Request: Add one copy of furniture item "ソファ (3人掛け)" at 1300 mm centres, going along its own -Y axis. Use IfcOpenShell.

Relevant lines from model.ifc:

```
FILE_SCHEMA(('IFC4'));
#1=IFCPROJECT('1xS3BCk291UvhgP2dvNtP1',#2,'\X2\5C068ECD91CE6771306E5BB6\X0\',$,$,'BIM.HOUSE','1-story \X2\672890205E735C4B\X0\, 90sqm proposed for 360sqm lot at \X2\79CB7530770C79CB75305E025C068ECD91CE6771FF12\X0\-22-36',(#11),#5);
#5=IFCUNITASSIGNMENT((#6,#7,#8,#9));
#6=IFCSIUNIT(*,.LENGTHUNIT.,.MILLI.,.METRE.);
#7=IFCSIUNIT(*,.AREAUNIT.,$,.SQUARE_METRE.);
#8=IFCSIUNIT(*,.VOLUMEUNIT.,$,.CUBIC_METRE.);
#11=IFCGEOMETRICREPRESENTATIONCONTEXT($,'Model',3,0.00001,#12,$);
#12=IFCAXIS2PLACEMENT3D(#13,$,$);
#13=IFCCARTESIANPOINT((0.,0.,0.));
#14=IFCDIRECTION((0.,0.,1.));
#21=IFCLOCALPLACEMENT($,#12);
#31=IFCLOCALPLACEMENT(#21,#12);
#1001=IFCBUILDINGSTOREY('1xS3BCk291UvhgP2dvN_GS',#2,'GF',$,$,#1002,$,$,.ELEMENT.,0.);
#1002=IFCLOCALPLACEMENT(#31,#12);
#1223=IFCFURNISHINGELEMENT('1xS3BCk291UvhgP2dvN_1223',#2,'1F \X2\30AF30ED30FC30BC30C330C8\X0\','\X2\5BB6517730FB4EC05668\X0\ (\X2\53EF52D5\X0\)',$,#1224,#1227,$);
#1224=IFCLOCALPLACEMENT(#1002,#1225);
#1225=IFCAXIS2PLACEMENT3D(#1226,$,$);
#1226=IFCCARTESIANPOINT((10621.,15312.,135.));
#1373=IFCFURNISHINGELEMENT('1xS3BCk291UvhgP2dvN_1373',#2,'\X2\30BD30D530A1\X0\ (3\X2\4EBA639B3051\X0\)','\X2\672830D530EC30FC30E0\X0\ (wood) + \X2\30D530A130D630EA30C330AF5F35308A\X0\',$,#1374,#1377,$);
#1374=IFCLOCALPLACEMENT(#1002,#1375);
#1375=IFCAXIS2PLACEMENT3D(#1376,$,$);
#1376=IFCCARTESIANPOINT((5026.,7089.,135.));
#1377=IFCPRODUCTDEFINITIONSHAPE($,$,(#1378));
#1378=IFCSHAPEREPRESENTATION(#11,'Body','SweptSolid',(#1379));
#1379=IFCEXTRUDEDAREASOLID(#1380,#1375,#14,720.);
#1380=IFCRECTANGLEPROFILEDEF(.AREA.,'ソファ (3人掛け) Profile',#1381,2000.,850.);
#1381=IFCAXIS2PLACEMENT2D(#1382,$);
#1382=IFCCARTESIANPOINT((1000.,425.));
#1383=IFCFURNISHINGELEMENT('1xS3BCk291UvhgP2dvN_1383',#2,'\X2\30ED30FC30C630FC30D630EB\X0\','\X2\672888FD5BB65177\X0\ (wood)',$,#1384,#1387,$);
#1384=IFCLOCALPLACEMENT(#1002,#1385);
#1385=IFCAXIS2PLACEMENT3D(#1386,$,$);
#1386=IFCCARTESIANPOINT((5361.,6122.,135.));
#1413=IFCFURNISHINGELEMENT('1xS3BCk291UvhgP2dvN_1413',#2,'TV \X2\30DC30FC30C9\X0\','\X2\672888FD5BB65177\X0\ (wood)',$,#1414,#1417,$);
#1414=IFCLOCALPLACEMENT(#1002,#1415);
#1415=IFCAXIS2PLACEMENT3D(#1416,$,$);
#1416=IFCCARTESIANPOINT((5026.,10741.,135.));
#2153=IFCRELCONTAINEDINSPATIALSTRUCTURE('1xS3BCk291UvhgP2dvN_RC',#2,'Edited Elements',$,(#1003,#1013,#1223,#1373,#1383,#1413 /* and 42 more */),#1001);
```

```python
import ifcopenshell
import ifcopenshell.api.geometry
import ifcopenshell.api.root
import ifcopenshell.util.element
import ifcopenshell.util.placement
import ifcopenshell.util.unit

model = ifcopenshell.open("model.ifc")
unit_scale = ifcopenshell.util.unit.calculate_unit_scale(model)


def reuse_history(source, copy):
    """copy_class also copies each property set's owner history, people and application; keep the originals."""
    for rel in copy.IsDefinedBy:
        if rel.is_a("IfcRelDefinesByProperties") and (history := rel.RelatingPropertyDefinition.OwnerHistory):
            rel.RelatingPropertyDefinition.OwnerHistory = source.OwnerHistory
            ifcopenshell.util.element.remove_deep2(model, history)


source = model.by_id(1373)
base = ifcopenshell.util.placement.get_local_placement(source.ObjectPlacement)
step = -base[:3, 1] * 1.3 / unit_scale

for i in range(1, 2):
    copy = ifcopenshell.api.root.copy_class(model, product=source)
    copy.Representation = ifcopenshell.util.element.copy_deep(
        model, source.Representation, exclude=["IfcGeometricRepresentationContext", "IfcRepresentationMap"]
    )
    reuse_history(source, copy)
    matrix = base.copy()
    matrix[:3, 3] += i * step
    print("added at", matrix[:3, 3].round(3) + 0.0)
    ifcopenshell.api.geometry.edit_object_placement(model, product=copy, matrix=matrix, is_si=False)

model.write("model_updated.ifc")
```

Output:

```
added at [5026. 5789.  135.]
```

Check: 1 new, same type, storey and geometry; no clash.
